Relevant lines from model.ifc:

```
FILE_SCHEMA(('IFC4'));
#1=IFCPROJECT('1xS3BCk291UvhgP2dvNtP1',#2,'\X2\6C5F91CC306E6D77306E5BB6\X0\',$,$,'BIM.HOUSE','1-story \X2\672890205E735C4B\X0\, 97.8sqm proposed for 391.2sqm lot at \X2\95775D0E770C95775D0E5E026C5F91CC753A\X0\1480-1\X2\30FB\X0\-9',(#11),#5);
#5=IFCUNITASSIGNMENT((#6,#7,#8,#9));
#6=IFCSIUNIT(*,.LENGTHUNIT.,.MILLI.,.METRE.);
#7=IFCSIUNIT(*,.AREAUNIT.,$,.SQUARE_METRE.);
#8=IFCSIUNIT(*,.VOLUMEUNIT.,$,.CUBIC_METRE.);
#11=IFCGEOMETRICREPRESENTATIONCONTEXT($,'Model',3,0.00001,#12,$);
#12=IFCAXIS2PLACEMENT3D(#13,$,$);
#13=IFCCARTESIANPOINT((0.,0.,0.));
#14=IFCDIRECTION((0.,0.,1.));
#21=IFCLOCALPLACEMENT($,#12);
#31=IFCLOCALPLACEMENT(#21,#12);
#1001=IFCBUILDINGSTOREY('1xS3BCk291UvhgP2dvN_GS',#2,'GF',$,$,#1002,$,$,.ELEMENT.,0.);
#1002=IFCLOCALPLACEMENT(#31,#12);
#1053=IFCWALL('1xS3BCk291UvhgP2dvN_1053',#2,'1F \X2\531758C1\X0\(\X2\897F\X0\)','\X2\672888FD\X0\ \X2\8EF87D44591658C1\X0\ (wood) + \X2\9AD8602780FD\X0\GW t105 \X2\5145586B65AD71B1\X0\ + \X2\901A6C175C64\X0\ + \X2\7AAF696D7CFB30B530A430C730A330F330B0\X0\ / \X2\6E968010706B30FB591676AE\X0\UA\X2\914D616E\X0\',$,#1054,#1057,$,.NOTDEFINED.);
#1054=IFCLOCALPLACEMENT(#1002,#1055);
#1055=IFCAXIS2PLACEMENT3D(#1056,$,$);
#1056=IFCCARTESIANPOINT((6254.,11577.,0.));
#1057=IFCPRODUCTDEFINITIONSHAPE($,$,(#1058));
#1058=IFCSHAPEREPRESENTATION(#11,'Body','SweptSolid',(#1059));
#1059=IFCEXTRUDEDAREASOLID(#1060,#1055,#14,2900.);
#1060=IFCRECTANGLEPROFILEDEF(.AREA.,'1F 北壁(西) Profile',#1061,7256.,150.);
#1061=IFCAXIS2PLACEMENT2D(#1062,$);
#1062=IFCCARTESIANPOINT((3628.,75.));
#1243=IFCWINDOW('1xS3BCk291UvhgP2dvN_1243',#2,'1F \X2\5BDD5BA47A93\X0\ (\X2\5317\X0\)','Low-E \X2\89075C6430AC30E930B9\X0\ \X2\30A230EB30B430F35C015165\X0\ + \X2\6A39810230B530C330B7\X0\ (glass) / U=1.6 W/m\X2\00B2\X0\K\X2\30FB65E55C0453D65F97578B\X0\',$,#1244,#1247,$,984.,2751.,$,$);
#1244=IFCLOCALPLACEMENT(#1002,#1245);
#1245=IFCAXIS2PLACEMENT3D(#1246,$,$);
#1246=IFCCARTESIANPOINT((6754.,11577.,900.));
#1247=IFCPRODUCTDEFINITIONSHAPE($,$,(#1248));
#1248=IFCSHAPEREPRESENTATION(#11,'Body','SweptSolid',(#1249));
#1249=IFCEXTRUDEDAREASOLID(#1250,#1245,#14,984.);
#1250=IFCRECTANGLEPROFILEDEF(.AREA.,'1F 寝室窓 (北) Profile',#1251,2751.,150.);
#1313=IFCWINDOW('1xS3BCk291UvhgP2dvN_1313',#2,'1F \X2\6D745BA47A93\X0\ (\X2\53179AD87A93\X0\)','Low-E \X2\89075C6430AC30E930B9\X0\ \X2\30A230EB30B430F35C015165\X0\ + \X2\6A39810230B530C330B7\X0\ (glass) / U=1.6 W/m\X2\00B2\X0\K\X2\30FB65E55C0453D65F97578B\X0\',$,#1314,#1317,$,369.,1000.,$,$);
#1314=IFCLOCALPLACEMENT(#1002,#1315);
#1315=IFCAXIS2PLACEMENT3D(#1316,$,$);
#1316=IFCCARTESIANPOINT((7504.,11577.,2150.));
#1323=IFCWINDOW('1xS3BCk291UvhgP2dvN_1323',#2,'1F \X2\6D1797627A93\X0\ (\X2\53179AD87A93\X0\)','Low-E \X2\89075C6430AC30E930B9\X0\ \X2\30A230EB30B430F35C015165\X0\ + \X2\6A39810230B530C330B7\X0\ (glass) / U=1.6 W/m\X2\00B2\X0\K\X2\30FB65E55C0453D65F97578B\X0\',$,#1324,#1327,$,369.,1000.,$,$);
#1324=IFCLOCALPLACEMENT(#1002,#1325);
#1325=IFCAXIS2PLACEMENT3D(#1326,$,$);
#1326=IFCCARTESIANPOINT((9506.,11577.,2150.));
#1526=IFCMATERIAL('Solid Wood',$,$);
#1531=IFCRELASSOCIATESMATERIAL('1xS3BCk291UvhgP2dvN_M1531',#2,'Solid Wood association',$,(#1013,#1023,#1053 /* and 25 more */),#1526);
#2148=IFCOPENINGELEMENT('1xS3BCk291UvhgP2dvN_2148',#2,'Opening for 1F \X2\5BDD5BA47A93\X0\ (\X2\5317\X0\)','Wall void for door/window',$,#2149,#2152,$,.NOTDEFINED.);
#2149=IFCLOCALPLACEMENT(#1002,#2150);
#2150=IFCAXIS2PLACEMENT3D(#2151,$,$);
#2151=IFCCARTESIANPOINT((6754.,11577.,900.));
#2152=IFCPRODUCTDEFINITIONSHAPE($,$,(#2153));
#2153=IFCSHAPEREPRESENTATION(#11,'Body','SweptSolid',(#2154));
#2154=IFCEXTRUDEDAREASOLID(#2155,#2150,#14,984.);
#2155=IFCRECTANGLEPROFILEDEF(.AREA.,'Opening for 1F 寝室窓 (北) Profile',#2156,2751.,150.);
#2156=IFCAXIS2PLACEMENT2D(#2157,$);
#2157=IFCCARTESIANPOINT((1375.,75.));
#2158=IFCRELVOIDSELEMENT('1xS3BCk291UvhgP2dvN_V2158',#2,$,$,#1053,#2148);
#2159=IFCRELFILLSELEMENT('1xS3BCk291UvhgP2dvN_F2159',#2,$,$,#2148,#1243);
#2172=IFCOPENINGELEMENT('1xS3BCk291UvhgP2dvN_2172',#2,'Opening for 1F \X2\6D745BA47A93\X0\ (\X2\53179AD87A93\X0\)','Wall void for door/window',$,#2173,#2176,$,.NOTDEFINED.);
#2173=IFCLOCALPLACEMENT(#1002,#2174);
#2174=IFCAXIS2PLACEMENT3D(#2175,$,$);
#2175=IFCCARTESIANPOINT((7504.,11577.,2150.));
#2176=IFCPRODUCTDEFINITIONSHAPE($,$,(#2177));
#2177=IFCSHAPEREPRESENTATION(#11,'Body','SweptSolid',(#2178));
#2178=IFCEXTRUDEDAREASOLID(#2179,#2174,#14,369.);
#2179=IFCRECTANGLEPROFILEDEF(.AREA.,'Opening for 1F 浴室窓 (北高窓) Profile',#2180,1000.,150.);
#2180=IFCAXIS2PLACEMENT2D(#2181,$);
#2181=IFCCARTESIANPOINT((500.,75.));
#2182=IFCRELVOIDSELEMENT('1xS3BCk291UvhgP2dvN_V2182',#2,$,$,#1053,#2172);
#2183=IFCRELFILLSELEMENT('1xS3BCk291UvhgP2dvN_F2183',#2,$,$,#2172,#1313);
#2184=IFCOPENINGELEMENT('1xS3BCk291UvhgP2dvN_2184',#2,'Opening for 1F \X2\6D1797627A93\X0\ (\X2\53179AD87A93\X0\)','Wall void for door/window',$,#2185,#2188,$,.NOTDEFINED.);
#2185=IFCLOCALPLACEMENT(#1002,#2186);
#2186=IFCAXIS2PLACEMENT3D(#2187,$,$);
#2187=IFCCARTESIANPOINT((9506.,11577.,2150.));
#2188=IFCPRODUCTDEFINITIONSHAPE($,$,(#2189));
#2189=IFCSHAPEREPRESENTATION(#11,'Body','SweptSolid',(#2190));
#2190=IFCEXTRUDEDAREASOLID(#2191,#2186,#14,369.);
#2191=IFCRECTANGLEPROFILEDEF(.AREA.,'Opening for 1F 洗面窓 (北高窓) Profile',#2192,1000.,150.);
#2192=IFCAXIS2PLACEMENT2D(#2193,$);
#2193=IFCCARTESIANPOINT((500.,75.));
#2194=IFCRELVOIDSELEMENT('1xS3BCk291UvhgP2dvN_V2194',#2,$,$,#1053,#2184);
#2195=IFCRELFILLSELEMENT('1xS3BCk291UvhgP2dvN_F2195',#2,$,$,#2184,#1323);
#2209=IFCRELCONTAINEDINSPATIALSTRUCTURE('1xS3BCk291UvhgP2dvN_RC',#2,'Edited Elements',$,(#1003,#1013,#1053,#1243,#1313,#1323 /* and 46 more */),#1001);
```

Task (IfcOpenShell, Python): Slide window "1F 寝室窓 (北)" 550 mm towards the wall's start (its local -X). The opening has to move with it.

```python
import ifcopenshell
import ifcopenshell.api.geometry
import ifcopenshell.util.placement

model = ifcopenshell.open("model.ifc")

window = model.by_guid("1xS3BCk291UvhgP2dvN_1243")
opening = window.FillsVoids[0].RelatingOpeningElement
wall = opening.VoidsElements[0].RelatingBuildingElement

wall_matrix = ifcopenshell.util.placement.get_local_placement(wall.ObjectPlacement)
shift = wall_matrix[:3, 0] * -550.0
before = ifcopenshell.util.placement.get_local_placement(window.ObjectPlacement)[:3, 3].copy()

# The window is not placed relative to its opening, so move both.
for product in (opening, window):
    matrix = ifcopenshell.util.placement.get_local_placement(product.ObjectPlacement)
    matrix[:3, 3] += shift
    ifcopenshell.api.geometry.edit_object_placement(model, product=product, matrix=matrix, is_si=False)

after = ifcopenshell.util.placement.get_local_placement(window.ObjectPlacement)[:3, 3]
print("window moved by", (after - before).round(3) + 0.0)

model.write("model_updated.ifc")
```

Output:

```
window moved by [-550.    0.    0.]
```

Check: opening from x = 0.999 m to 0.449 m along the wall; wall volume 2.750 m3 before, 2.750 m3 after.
